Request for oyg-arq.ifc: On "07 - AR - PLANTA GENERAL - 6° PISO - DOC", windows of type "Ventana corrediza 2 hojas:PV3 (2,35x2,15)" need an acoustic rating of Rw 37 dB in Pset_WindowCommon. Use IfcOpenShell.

First a look at what the model holds.

```python
import ifcopenshell
import ifcopenshell.util.element

model = ifcopenshell.open("oyg-arq.ifc")
print(model.schema)
storey = next(s for s in model.by_type("IfcBuildingStorey") if s.Name == "07 - AR - PLANTA GENERAL - 6° PISO - DOC")
windows = [e for e in ifcopenshell.util.element.get_decomposition(storey) if e.is_a("IfcWindow")]
seen = {}
for e in windows:
    element_type = ifcopenshell.util.element.get_type(e)
    key = (element_type.Name if element_type != e and element_type else None, ifcopenshell.util.element.get_pset(e, "Pset_WindowCommon", "AcousticRating"))
    seen[key] = seen.get(key, 0) + 1
for (name, value), count in sorted(seen.items(), key=str):
    print(count, "x", name, "|", value)
```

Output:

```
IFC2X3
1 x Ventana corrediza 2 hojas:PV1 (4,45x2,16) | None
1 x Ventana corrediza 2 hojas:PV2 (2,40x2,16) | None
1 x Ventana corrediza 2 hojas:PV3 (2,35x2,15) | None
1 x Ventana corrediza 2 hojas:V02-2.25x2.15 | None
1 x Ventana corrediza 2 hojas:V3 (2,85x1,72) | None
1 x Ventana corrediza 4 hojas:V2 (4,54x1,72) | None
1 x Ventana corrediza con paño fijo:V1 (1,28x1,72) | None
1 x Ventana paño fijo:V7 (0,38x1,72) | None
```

```python
import ifcopenshell
import ifcopenshell.api.pset
import ifcopenshell.util.element

model = ifcopenshell.open("oyg-arq.ifc")

storey = next(s for s in model.by_type("IfcBuildingStorey") if s.Name == "07 - AR - PLANTA GENERAL - 6° PISO - DOC")
windows = [e for e in ifcopenshell.util.element.get_decomposition(storey) if e.is_a("IfcWindow")]

count = 0
for e in windows:
    element_type = ifcopenshell.util.element.get_type(e)
    if element_type in (None, e) or element_type.Name != "Ventana corrediza 2 hojas:PV3 (2,35x2,15)":
        continue
    # add_pset returns the element's existing set when there is one.
    pset = ifcopenshell.api.pset.add_pset(model, product=e, name="Pset_WindowCommon")
    ifcopenshell.api.pset.edit_pset(model, pset=pset, properties={"AcousticRating": "Rw 37 dB"})
    count += 1

print(count, "windows updated")

model.write("oyg-arq_rev.ifc")
```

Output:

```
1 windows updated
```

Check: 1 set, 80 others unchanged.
